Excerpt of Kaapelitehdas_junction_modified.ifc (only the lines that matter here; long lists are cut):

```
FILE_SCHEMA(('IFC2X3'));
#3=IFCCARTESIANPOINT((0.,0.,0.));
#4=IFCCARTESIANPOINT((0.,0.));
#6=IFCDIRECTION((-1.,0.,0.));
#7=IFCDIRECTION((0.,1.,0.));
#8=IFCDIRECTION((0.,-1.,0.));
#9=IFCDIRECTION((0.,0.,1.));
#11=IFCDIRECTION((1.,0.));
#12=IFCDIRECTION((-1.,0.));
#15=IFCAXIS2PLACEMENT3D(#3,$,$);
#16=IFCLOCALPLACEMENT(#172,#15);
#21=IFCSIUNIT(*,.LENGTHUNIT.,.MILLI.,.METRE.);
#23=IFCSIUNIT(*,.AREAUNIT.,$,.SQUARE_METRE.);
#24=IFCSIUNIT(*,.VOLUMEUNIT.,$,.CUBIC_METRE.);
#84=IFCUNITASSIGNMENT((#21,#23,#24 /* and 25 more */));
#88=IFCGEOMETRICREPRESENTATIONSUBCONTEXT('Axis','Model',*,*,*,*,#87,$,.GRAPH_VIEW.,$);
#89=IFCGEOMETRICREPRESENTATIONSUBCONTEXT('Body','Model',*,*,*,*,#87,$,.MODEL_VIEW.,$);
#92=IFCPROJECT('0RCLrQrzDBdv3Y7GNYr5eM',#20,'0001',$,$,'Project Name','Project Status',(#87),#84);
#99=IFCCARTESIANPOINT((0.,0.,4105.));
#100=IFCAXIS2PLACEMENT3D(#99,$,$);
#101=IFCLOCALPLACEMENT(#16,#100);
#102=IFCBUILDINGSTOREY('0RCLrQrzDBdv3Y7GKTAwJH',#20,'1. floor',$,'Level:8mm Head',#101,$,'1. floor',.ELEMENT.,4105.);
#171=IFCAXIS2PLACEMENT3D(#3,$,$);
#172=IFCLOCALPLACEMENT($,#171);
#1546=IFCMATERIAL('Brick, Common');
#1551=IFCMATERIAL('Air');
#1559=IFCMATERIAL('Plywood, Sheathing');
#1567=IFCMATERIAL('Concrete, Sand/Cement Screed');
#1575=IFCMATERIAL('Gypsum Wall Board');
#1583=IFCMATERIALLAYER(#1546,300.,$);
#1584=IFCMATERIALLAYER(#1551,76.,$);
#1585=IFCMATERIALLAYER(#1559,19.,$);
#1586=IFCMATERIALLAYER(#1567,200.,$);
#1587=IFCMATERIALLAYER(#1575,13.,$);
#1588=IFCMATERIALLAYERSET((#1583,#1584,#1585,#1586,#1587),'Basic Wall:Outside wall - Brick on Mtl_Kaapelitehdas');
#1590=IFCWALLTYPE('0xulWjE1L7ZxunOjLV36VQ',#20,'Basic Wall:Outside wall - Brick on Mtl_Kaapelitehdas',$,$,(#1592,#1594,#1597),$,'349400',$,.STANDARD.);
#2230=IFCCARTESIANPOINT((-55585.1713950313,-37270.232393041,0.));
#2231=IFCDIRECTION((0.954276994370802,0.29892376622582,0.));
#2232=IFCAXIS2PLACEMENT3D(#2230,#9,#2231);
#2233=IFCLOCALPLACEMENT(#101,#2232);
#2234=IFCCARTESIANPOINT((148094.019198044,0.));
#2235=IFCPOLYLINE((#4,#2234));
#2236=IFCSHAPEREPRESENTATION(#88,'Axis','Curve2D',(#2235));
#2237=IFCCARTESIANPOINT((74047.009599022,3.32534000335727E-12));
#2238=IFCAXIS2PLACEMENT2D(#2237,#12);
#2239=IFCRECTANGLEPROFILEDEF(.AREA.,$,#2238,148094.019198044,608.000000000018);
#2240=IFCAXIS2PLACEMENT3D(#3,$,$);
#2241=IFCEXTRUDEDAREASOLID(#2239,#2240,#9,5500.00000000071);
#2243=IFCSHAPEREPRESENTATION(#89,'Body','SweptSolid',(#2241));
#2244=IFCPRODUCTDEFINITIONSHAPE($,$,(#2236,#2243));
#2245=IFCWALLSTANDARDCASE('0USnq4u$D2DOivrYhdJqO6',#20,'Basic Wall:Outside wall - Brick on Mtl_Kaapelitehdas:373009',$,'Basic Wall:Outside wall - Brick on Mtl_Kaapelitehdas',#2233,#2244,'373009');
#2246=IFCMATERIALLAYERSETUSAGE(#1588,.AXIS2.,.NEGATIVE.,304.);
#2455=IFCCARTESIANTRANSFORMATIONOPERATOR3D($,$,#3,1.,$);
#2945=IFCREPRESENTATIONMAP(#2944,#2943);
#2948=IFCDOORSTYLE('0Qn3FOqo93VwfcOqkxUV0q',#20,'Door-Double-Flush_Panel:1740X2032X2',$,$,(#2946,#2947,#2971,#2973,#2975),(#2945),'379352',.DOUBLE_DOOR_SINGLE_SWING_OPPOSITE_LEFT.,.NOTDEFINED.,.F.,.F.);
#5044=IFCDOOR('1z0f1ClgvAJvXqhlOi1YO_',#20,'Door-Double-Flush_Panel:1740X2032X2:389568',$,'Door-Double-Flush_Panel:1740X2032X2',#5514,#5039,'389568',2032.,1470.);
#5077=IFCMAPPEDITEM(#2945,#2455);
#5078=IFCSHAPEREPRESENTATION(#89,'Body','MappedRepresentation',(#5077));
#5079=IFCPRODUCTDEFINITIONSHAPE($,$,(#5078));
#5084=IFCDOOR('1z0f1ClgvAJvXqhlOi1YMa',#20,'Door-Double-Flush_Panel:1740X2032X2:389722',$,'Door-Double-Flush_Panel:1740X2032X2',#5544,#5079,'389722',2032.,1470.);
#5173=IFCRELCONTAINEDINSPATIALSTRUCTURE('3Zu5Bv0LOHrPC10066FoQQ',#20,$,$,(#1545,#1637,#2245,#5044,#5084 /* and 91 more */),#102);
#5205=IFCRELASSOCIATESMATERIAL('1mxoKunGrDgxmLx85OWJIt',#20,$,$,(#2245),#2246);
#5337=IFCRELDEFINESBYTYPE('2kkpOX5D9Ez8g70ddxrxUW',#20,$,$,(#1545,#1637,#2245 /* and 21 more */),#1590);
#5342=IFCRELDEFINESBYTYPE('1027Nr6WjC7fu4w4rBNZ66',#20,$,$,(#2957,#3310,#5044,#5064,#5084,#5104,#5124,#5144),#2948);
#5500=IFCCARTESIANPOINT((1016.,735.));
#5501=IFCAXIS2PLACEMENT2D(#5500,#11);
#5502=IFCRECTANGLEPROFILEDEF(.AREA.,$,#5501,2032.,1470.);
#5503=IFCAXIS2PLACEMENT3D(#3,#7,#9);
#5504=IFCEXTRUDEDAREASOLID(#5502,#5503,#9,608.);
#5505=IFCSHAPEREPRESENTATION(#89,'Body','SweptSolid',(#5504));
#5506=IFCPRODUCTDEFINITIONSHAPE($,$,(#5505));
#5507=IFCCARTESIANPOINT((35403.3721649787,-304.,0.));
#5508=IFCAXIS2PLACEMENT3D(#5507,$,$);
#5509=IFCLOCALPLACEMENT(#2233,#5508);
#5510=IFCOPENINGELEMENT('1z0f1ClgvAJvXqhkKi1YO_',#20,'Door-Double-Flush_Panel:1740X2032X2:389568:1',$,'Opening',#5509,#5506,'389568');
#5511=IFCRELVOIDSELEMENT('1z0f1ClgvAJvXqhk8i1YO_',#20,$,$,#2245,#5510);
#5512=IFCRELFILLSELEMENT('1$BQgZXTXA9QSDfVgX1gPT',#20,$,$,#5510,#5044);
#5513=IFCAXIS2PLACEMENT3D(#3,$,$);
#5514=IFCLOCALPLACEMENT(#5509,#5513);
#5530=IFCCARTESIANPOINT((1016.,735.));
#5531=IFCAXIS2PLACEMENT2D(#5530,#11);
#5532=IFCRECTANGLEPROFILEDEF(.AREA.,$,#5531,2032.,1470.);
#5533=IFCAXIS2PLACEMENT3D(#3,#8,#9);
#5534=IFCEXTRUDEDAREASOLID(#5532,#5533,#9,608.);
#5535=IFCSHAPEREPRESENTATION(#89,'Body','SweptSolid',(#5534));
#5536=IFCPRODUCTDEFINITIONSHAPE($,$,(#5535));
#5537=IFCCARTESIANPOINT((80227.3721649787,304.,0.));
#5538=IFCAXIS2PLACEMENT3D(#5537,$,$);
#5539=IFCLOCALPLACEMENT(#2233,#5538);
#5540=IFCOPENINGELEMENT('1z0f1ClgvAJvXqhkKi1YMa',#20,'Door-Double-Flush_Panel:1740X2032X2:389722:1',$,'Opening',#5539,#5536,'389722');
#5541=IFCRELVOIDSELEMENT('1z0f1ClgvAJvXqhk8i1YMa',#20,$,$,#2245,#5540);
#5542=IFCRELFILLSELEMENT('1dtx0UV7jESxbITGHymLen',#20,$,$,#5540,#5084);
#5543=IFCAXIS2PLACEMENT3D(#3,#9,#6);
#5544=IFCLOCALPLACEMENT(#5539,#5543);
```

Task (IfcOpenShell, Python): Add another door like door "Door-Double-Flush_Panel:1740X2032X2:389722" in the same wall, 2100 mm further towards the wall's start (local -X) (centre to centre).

```python
import ifcopenshell
import ifcopenshell.api.feature
import ifcopenshell.api.geometry
import ifcopenshell.api.root
import ifcopenshell.geom
import ifcopenshell.util.element
import ifcopenshell.util.placement
import ifcopenshell.util.shape
import ifcopenshell.util.unit

model = ifcopenshell.open("Kaapelitehdas_junction_modified.ifc")
unit_scale = ifcopenshell.util.unit.calculate_unit_scale(model)
settings = ifcopenshell.geom.settings()


def volume(element):
    """Net volume in cubic metres, openings subtracted."""
    shape = ifcopenshell.geom.create_shape(settings, element)
    return ifcopenshell.util.shape.get_volume(shape.geometry)


def reuse_history(source, copy):
    """copy_class also copies each property set's owner history, people and application; keep the originals."""
    for rel in copy.IsDefinedBy:
        if rel.is_a("IfcRelDefinesByProperties") and (history := rel.RelatingPropertyDefinition.OwnerHistory):
            rel.RelatingPropertyDefinition.OwnerHistory = source.OwnerHistory
            ifcopenshell.util.element.remove_deep2(model, history)


door = model.by_guid("1z0f1ClgvAJvXqhlOi1YMa")
opening = door.FillsVoids[0].RelatingOpeningElement
wall = opening.VoidsElements[0].RelatingBuildingElement
before = volume(wall)
shift = ifcopenshell.util.placement.get_local_placement(wall.ObjectPlacement)[:3, 0] * -2.1 / unit_scale

# copy_class copies the void relationship, type, container and properties, but no geometry.
new_opening = ifcopenshell.api.root.copy_class(model, product=opening)
new_opening.Representation = ifcopenshell.util.element.copy_deep(
    model, opening.Representation, exclude=["IfcGeometricRepresentationContext", "IfcRepresentationMap"]
)
new_opening.Name = "Door-Double-Flush_Panel:1740X2032X2"
new_opening.Tag = None
new_door = ifcopenshell.api.root.copy_class(model, product=door)
new_door.Representation = ifcopenshell.util.element.copy_deep(
    model, door.Representation, exclude=["IfcGeometricRepresentationContext", "IfcRepresentationMap"]
)
new_door.Name = "Door-Double-Flush_Panel:1740X2032X2"
new_door.Tag = None
reuse_history(door, new_door)
fills = ifcopenshell.api.feature.add_filling(model, opening=new_opening, element=new_door)
fills.OwnerHistory = new_door.OwnerHistory  # required in IFC2X3

for old, new in ((opening, new_opening), (door, new_door)):
    matrix = ifcopenshell.util.placement.get_local_placement(old.ObjectPlacement)
    matrix[:3, 3] += shift
    ifcopenshell.api.geometry.edit_object_placement(model, product=new, matrix=matrix, is_si=False)

after = volume(wall)

print(f"wall volume {before:.3f} -> {after:.3f} m3")

model.write("Kaapelitehdas_junction_modified_v2.ifc")
```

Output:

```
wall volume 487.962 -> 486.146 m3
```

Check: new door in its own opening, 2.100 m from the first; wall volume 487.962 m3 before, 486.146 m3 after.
